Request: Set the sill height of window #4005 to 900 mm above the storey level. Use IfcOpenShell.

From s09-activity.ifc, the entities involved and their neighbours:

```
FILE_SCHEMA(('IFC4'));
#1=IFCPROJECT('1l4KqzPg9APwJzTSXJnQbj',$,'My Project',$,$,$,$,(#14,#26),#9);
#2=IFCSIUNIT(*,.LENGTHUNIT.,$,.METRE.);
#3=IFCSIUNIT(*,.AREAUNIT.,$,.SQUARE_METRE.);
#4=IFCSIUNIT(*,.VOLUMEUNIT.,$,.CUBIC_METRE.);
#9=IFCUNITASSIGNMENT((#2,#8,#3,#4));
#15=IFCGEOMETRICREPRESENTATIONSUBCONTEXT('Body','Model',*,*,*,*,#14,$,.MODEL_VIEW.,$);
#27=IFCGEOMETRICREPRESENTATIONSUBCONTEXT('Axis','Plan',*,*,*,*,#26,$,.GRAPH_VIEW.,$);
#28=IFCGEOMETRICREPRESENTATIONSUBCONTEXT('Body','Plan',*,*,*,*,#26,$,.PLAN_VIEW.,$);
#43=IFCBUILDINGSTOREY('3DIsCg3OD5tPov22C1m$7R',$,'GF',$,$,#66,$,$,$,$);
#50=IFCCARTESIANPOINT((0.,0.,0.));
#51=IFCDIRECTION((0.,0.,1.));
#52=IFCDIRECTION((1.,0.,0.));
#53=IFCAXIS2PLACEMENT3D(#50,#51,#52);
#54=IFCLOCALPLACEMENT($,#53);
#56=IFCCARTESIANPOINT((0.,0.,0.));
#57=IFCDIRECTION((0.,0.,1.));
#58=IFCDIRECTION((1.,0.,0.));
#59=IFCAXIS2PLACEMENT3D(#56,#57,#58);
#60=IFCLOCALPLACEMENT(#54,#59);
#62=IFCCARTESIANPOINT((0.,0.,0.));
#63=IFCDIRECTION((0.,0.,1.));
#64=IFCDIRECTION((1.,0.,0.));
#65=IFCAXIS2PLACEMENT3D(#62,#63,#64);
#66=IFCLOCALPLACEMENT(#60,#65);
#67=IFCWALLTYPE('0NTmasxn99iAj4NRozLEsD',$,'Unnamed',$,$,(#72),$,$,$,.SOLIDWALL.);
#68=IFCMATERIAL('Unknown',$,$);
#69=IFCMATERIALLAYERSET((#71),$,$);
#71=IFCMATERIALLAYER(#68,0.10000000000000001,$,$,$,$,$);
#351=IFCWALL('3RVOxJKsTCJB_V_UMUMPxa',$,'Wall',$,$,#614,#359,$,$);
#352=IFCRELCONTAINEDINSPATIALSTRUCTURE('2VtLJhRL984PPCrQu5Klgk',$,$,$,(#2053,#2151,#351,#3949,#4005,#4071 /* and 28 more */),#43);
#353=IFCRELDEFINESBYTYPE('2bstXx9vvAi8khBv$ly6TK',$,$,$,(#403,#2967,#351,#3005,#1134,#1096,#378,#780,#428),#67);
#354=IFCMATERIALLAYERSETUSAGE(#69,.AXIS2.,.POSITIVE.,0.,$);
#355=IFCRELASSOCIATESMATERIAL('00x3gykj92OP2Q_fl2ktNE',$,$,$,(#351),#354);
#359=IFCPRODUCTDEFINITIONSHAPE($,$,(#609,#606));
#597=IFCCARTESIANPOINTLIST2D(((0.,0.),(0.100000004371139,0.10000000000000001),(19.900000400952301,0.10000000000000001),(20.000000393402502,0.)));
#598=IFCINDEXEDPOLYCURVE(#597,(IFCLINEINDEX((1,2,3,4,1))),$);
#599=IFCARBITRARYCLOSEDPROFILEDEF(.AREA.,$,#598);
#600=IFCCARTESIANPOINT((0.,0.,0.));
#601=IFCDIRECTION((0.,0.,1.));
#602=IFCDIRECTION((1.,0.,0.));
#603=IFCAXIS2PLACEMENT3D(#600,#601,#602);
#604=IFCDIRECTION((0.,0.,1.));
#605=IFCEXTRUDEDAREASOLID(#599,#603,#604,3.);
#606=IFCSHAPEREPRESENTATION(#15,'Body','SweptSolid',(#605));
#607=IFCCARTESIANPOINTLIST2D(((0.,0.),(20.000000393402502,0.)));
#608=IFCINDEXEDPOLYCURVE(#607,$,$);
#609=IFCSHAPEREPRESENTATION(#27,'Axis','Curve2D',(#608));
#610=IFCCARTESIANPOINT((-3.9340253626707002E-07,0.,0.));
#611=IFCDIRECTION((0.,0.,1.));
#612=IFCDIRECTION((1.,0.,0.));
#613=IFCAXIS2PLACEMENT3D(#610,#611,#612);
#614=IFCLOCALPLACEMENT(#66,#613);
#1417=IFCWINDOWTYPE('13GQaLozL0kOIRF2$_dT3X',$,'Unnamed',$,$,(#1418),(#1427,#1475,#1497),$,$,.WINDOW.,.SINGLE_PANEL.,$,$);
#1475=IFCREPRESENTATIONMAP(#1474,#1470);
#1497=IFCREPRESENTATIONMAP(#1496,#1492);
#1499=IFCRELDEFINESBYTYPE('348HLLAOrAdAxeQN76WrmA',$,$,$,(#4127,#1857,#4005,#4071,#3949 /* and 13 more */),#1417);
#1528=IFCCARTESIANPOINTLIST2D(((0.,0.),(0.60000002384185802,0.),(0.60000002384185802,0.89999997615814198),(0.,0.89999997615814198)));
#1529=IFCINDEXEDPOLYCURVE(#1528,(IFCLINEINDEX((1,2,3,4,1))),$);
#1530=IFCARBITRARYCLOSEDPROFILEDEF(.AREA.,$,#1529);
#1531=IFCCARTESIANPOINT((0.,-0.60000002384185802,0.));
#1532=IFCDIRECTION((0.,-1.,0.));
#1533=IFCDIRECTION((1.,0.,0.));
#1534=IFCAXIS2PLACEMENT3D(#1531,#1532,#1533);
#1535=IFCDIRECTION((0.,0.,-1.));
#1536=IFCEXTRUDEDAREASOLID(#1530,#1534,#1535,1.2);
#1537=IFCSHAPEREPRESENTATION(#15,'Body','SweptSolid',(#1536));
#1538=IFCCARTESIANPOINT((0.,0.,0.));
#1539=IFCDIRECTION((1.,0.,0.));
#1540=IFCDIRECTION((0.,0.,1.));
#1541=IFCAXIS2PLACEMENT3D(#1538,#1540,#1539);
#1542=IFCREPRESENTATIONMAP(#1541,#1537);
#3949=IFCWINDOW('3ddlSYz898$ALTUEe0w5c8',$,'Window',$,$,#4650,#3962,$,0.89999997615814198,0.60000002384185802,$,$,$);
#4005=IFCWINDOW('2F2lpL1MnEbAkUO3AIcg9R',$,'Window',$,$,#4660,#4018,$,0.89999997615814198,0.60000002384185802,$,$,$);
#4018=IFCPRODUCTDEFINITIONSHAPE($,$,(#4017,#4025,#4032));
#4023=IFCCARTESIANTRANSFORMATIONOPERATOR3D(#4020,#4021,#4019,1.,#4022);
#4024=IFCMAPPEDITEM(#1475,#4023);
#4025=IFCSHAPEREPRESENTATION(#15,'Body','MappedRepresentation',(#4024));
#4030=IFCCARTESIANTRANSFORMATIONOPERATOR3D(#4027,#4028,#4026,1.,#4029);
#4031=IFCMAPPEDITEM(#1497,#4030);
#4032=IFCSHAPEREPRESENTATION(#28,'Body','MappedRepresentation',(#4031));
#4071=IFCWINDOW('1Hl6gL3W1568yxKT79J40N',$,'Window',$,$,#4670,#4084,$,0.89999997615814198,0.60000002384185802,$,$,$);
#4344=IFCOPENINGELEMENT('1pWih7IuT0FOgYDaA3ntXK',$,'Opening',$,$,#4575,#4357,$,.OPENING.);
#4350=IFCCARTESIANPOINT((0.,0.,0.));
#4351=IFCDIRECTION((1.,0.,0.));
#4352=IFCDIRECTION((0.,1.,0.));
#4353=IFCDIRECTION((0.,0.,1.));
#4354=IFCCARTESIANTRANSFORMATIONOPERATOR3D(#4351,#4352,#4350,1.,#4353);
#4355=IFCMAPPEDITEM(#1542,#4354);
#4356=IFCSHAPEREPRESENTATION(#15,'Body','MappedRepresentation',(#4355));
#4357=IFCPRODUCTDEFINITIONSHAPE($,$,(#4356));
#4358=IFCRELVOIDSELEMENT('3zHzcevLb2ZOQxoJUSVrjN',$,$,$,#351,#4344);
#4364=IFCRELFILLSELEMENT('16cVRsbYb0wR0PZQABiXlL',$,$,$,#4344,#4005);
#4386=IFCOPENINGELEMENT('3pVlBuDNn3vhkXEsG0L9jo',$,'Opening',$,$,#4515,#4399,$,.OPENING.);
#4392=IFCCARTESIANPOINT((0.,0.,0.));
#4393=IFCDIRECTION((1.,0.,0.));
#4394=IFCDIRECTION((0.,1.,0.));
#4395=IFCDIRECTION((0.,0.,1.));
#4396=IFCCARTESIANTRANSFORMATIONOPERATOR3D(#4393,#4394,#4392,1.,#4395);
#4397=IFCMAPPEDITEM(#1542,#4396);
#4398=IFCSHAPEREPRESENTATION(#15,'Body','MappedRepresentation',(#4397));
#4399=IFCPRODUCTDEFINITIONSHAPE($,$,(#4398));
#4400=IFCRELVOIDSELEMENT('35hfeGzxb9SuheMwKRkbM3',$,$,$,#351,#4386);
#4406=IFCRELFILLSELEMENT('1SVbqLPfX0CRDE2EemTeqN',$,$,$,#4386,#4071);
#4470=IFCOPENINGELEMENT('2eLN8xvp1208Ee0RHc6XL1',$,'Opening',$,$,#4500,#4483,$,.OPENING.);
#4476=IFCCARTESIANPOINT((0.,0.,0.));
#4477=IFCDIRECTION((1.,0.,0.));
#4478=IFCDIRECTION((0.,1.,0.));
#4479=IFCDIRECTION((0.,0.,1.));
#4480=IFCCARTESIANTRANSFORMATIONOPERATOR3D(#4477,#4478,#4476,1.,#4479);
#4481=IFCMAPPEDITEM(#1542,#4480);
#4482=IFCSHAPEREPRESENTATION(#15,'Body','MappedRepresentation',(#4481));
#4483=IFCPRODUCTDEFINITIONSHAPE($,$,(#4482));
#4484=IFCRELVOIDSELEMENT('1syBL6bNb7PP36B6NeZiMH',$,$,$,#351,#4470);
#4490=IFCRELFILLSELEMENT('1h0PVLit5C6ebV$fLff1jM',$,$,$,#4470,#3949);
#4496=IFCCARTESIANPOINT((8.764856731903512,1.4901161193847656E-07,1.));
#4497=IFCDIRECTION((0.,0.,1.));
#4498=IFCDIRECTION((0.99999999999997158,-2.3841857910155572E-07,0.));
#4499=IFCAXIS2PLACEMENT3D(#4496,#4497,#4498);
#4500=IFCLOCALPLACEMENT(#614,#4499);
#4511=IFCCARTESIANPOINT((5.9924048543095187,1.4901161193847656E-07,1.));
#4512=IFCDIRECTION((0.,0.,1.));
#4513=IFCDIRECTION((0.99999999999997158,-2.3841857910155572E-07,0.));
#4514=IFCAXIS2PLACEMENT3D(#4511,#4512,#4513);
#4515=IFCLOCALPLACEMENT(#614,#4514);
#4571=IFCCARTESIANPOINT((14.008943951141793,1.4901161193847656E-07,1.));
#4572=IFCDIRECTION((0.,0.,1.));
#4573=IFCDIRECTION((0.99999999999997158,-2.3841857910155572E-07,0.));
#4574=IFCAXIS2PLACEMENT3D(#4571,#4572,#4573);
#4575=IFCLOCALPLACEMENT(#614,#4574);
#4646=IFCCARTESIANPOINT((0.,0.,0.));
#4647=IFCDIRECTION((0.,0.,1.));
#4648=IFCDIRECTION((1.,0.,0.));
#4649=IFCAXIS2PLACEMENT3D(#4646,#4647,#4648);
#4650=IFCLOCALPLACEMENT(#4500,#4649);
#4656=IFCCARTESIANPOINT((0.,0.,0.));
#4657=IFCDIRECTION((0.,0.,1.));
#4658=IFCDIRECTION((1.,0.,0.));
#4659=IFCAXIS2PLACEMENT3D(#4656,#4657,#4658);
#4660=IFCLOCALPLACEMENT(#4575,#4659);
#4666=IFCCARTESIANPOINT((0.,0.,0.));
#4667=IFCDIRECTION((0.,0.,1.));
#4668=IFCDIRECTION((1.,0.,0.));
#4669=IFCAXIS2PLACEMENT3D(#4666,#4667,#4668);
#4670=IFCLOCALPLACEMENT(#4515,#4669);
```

```python
import numpy as np
import ifcopenshell
import ifcopenshell.api.geometry
import ifcopenshell.geom
import ifcopenshell.util.element
import ifcopenshell.util.placement
import ifcopenshell.util.shape
import ifcopenshell.util.unit

model = ifcopenshell.open("s09-activity.ifc")
unit_scale = ifcopenshell.util.unit.calculate_unit_scale(model)

window = model.by_id(4005)
opening = window.FillsVoids[0].RelatingOpeningElement
storey = ifcopenshell.util.element.get_container(window, ifc_class="IfcBuildingStorey")
level = ifcopenshell.util.placement.get_local_placement(storey.ObjectPlacement)[2, 3]

# The opening's origin need not be at the sill, so measure its lowest point.
shape = ifcopenshell.geom.create_shape(ifcopenshell.geom.settings(), opening)
bottom = ifcopenshell.util.shape.get_shape_bottom_elevation(shape, shape.geometry) / unit_scale
dz = level + 0.9 / unit_scale - bottom

shift = np.array([0.0, 0.0, dz])
# The window is placed relative to its opening, so it follows when the opening moves.
matrix = ifcopenshell.util.placement.get_local_placement(opening.ObjectPlacement)
matrix[:3, 3] += shift
ifcopenshell.api.geometry.edit_object_placement(
    model, product=opening, matrix=matrix, is_si=False, should_transform_children=True
)

print(f"moved by {dz * unit_scale:+.3f} m")

model.write("s09-activity_updated.ifc")
```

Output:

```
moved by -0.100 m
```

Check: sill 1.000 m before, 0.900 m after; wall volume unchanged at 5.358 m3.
